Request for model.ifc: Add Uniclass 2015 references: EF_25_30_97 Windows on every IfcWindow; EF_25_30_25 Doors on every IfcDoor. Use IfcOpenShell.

First a look at what the model holds.

```python
import ifcopenshell

model = ifcopenshell.open("model.ifc")
print(model.schema)
print("classifications:", [c.Name for c in model.by_type("IfcClassification")])
for ifc_class in ("IfcDoor", "IfcRoof", "IfcStair", "IfcWall", "IfcWindow"):
    print(ifc_class, len(model.by_type(ifc_class)))
```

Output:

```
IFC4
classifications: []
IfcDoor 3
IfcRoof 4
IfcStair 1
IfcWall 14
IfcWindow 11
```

```python
import ifcopenshell
import ifcopenshell.api.classification

model = ifcopenshell.open("model.ifc")

system = ifcopenshell.api.classification.add_classification(model, classification="Uniclass 2015")

codes = {
    "IfcWindow": ("EF_25_30_97", "Windows"),
    "IfcDoor": ("EF_25_30_25", "Doors"),
}
for ifc_class, (code, name) in codes.items():
    products = model.by_type(ifc_class)
    ifcopenshell.api.classification.add_reference(
        model, products=products, classification=system, identification=code, name=name
    )
    print(code, len(products))

model.write("model_rev.ifc")
```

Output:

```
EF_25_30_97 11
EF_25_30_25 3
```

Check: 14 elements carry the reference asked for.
